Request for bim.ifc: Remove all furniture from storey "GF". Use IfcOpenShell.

First a look at what the model holds.

```python
import ifcopenshell
import ifcopenshell.util.element

model = ifcopenshell.open("bim.ifc")
print(model.schema)
storey = next(s for s in model.by_type("IfcBuildingStorey") if s.Name == "GF")
furniture = [e for e in ifcopenshell.util.element.get_decomposition(storey) if e.is_a("IfcFurnishingElement")]
seen = {}
for e in furniture:
    element_type = ifcopenshell.util.element.get_type(e)
    name = element_type.Name if element_type not in (None, e) else None
    seen[name] = seen.get(name, 0) + 1
for name, count in sorted(seen.items(), key=str):
    print(count, "x", name)
```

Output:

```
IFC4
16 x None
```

```python
import ifcopenshell
import ifcopenshell.api.root
import ifcopenshell.util.element

model = ifcopenshell.open("bim.ifc")

storey = next(s for s in model.by_type("IfcBuildingStorey") if s.Name == "GF")
furniture = [e for e in ifcopenshell.util.element.get_decomposition(storey) if e.is_a("IfcFurnishingElement")]

for e in furniture:
    ifcopenshell.api.root.remove_product(model, product=e)
print(len(furniture), "removed")

model.write("bim_updated.ifc")
```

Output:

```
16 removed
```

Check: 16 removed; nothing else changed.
